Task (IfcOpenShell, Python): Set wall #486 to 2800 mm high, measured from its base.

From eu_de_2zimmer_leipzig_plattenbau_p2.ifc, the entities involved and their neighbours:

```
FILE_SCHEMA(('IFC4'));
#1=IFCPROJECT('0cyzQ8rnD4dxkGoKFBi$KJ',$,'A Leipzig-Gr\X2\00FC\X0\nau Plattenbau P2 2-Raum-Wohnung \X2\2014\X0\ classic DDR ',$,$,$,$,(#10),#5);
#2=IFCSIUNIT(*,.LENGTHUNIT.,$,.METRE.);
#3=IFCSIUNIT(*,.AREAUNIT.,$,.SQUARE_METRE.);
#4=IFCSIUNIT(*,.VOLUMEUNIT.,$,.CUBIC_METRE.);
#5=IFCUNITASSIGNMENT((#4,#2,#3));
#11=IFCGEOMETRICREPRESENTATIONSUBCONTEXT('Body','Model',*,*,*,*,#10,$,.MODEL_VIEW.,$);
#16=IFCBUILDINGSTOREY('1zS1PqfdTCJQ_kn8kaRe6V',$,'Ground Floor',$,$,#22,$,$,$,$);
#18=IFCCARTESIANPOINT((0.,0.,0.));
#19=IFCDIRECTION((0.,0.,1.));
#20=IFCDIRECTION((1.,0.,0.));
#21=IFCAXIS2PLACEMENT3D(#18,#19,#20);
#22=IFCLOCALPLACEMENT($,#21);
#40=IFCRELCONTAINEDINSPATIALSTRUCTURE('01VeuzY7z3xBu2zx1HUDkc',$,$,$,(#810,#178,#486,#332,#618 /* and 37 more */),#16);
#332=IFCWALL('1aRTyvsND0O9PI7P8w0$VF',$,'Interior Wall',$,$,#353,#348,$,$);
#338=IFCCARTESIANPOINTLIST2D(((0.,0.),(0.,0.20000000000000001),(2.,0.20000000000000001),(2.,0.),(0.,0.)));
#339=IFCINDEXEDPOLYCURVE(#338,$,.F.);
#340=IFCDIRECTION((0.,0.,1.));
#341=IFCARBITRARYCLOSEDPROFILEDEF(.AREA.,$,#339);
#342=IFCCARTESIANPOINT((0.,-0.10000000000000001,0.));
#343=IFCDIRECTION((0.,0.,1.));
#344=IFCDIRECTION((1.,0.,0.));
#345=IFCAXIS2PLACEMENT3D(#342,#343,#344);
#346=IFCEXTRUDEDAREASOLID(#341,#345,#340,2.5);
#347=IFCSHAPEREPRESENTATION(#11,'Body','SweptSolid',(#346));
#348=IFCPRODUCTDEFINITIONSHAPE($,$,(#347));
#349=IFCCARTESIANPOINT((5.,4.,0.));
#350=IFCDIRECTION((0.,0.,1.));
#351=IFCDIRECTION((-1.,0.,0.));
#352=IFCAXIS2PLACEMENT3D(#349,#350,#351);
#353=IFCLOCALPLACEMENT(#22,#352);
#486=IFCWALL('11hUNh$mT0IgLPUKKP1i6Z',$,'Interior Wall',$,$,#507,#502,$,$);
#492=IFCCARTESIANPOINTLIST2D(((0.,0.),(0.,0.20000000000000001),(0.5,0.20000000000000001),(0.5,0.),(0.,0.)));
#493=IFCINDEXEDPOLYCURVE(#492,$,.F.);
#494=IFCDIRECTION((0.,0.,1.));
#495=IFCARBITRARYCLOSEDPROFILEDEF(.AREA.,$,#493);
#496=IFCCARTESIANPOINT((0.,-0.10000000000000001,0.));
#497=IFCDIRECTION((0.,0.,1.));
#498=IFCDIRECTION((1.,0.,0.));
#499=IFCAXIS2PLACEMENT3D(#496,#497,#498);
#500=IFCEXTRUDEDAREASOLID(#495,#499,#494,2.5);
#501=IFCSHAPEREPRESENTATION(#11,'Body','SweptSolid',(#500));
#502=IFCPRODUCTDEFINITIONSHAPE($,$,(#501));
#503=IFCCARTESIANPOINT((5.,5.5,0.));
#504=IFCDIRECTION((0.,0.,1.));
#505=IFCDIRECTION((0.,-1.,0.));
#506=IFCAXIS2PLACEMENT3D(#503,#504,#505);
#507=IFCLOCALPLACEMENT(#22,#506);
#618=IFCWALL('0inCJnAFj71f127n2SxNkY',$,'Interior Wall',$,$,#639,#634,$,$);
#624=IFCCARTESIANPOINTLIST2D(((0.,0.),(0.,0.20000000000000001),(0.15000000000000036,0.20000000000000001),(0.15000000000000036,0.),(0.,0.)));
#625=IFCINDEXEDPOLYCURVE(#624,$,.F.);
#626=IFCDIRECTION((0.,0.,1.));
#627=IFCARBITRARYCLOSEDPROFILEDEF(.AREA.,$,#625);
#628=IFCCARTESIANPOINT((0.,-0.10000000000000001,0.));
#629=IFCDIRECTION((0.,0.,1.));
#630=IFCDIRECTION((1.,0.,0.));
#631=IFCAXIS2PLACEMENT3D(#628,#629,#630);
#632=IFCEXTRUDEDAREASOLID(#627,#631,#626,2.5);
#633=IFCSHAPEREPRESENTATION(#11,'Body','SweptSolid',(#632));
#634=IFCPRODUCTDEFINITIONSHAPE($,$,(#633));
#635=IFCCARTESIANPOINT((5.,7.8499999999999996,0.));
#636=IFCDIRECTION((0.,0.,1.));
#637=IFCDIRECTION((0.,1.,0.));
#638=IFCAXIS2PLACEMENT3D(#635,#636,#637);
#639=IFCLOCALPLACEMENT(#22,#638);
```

```python
import ifcopenshell
import ifcopenshell.geom
import ifcopenshell.util.representation
import ifcopenshell.util.shape
import ifcopenshell.util.unit

model = ifcopenshell.open("eu_de_2zimmer_leipzig_plattenbau_p2.ifc")
unit_scale = ifcopenshell.util.unit.calculate_unit_scale(model)
settings = ifcopenshell.geom.settings()


def volume(element):
    """Net volume in cubic metres, openings subtracted."""
    shape = ifcopenshell.geom.create_shape(settings, element)
    return ifcopenshell.util.shape.get_volume(shape.geometry)


wall = model.by_guid("11hUNh$mT0IgLPUKKP1i6Z")
before = volume(wall)

body = ifcopenshell.util.representation.get_representation(wall, "Model", "Body")
solid = body.Items[0]
old_height = solid.Depth
solid.Depth = 2.8 / unit_scale
after = volume(wall)

print(f"height {old_height:g} -> {solid.Depth:g}, volume {before:.3f} -> {after:.3f} m3")

model.write("eu_de_2zimmer_leipzig_plattenbau_p2_edited.ifc")
```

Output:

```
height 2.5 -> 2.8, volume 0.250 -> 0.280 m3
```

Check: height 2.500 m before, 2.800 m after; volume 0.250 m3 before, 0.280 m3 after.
